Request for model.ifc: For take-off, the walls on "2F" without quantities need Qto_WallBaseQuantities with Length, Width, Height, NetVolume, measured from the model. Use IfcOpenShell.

First a look at what the model holds.

```python
import ifcopenshell
import ifcopenshell.util.element
import ifcopenshell.util.unit

model = ifcopenshell.open("model.ifc")
print(model.schema)
for unit_type in ("LENGTHUNIT", "AREAUNIT", "VOLUMEUNIT"):
    print(unit_type, ifcopenshell.util.unit.calculate_unit_scale(model, unit_type))
storey = next(s for s in model.by_type("IfcBuildingStorey") if s.Name == "2F")
walls = [e for e in ifcopenshell.util.element.get_decomposition(storey) if e.is_a("IfcWall")]
for e in sorted(walls, key=lambda e: e.id()):
    print(e.id(), e.is_a(), e.Name, list(ifcopenshell.util.element.get_psets(e, qtos_only=True)), sep=" | ")
```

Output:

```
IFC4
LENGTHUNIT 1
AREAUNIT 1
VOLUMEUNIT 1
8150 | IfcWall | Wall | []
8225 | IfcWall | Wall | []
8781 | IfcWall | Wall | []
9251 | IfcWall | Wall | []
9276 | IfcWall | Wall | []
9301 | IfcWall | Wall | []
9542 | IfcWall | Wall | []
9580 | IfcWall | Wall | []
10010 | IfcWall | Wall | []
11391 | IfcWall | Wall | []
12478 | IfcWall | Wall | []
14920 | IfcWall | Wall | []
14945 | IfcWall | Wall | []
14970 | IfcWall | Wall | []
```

```python
import ifcopenshell
import ifcopenshell.api.pset
import ifcopenshell.geom
import ifcopenshell.util.element
import ifcopenshell.util.shape
import ifcopenshell.util.unit

model = ifcopenshell.open("model.ifc")
unit_scale = ifcopenshell.util.unit.calculate_unit_scale(model)
volume_scale = ifcopenshell.util.unit.calculate_unit_scale(model, "VOLUMEUNIT")
settings = ifcopenshell.geom.settings()

storey = next(s for s in model.by_type("IfcBuildingStorey") if s.Name == "2F")
walls = [e for e in ifcopenshell.util.element.get_decomposition(storey) if e.is_a("IfcWall")]

for e in sorted(walls, key=lambda e: e.id()):
    if ifcopenshell.util.element.get_psets(e, qtos_only=True, should_inherit=False):
        continue
    # Geometry comes back in metres, in the element's own axes.
    shape = ifcopenshell.geom.create_shape(settings, e)
    values = {
        "Length": ifcopenshell.util.shape.get_x(shape.geometry) / unit_scale,
        "Width": ifcopenshell.util.shape.get_y(shape.geometry) / unit_scale,
        "Height": ifcopenshell.util.shape.get_z(shape.geometry) / unit_scale,
        "NetVolume": ifcopenshell.util.shape.get_volume(shape.geometry) / volume_scale,
    }
    qto = ifcopenshell.api.pset.add_qto(model, product=e, name="Qto_WallBaseQuantities")
    ifcopenshell.api.pset.edit_qto(model, qto=qto, properties=values)
    print(e.id(), {k: round(v, 3) for k, v in values.items()})

model.write("model_v2.ifc")
```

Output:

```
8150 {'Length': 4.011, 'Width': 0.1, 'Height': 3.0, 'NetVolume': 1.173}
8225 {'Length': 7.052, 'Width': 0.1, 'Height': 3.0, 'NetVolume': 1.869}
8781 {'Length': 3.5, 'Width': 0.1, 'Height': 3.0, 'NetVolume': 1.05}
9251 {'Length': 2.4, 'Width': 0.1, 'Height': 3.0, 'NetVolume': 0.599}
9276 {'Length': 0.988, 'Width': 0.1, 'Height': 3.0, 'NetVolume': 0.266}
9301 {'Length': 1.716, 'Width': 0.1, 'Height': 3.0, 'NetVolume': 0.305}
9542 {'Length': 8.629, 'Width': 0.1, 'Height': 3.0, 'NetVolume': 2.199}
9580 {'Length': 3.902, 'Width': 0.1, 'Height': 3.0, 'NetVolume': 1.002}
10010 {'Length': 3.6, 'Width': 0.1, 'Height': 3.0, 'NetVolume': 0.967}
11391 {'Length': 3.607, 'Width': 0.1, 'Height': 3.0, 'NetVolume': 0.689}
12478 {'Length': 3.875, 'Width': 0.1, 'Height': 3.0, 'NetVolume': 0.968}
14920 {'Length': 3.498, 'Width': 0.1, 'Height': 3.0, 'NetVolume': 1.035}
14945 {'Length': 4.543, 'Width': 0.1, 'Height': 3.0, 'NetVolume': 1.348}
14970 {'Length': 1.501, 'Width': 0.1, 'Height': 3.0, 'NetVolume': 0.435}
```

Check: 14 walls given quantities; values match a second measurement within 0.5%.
